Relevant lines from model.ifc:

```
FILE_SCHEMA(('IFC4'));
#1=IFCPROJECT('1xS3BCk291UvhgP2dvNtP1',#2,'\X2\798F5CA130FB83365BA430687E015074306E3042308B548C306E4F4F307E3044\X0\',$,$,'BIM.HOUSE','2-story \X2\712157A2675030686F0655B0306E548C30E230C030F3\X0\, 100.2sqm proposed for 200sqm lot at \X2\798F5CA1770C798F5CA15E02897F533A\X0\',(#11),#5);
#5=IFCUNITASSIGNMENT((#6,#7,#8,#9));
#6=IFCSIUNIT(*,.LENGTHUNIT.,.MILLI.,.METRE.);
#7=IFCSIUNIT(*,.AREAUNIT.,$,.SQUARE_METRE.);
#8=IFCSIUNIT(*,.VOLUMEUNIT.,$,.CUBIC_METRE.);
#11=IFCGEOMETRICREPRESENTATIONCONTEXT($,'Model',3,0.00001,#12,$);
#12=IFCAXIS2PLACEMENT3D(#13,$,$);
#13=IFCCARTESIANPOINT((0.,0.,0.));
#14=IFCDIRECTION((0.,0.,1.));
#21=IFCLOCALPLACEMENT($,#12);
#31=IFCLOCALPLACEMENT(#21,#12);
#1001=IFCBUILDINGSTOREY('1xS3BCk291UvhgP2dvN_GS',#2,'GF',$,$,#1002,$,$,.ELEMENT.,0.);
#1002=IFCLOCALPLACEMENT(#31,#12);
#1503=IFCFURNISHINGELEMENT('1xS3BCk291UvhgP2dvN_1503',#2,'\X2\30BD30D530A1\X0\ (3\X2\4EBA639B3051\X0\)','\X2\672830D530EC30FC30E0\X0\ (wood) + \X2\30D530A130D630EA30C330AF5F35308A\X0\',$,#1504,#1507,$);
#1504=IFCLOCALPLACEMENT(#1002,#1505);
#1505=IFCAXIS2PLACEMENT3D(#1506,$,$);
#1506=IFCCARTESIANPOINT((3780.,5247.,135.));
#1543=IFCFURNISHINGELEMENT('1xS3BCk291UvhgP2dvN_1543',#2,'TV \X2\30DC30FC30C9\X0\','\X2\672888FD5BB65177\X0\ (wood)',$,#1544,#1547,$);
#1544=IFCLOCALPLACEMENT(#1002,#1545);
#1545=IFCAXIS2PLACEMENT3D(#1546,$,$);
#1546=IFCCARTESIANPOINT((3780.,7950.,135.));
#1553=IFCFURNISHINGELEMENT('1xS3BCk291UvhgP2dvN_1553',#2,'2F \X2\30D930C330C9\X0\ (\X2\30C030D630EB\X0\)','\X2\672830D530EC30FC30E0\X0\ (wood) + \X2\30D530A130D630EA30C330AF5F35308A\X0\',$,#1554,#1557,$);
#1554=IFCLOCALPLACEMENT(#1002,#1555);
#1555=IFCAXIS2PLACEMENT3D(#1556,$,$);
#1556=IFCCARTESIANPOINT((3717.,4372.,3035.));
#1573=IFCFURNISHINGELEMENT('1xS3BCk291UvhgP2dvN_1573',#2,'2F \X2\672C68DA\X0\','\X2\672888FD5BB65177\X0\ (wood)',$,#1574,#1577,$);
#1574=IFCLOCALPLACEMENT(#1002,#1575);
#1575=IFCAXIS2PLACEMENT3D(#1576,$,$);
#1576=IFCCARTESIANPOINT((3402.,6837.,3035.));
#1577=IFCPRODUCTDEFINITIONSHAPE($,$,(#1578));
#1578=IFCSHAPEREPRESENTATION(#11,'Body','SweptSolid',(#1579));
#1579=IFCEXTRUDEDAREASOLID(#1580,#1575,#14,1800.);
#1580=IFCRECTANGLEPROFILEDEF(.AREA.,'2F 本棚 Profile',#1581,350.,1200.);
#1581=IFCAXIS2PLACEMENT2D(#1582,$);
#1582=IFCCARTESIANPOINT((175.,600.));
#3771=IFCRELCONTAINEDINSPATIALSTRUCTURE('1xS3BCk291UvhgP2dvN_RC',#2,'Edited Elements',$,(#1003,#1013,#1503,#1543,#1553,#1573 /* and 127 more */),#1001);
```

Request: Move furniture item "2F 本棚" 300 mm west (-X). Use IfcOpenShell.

```python
import ifcopenshell
import ifcopenshell.api.geometry
import ifcopenshell.util.placement
import ifcopenshell.util.unit

model = ifcopenshell.open("model.ifc")
unit_scale = ifcopenshell.util.unit.calculate_unit_scale(model)

item = model.by_guid("1xS3BCk291UvhgP2dvN_1573")
matrix = ifcopenshell.util.placement.get_local_placement(item.ObjectPlacement)
matrix[0, 3] -= 0.3 / unit_scale
ifcopenshell.api.geometry.edit_object_placement(model, product=item, matrix=matrix, is_si=False)

print(ifcopenshell.util.placement.get_local_placement(item.ObjectPlacement).round(3) + 0.0)

model.write("model_v2.ifc")
```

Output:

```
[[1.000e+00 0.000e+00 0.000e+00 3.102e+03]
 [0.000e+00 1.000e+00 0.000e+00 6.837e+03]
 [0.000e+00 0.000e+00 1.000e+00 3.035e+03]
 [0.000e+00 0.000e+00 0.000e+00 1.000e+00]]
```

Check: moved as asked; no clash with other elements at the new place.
